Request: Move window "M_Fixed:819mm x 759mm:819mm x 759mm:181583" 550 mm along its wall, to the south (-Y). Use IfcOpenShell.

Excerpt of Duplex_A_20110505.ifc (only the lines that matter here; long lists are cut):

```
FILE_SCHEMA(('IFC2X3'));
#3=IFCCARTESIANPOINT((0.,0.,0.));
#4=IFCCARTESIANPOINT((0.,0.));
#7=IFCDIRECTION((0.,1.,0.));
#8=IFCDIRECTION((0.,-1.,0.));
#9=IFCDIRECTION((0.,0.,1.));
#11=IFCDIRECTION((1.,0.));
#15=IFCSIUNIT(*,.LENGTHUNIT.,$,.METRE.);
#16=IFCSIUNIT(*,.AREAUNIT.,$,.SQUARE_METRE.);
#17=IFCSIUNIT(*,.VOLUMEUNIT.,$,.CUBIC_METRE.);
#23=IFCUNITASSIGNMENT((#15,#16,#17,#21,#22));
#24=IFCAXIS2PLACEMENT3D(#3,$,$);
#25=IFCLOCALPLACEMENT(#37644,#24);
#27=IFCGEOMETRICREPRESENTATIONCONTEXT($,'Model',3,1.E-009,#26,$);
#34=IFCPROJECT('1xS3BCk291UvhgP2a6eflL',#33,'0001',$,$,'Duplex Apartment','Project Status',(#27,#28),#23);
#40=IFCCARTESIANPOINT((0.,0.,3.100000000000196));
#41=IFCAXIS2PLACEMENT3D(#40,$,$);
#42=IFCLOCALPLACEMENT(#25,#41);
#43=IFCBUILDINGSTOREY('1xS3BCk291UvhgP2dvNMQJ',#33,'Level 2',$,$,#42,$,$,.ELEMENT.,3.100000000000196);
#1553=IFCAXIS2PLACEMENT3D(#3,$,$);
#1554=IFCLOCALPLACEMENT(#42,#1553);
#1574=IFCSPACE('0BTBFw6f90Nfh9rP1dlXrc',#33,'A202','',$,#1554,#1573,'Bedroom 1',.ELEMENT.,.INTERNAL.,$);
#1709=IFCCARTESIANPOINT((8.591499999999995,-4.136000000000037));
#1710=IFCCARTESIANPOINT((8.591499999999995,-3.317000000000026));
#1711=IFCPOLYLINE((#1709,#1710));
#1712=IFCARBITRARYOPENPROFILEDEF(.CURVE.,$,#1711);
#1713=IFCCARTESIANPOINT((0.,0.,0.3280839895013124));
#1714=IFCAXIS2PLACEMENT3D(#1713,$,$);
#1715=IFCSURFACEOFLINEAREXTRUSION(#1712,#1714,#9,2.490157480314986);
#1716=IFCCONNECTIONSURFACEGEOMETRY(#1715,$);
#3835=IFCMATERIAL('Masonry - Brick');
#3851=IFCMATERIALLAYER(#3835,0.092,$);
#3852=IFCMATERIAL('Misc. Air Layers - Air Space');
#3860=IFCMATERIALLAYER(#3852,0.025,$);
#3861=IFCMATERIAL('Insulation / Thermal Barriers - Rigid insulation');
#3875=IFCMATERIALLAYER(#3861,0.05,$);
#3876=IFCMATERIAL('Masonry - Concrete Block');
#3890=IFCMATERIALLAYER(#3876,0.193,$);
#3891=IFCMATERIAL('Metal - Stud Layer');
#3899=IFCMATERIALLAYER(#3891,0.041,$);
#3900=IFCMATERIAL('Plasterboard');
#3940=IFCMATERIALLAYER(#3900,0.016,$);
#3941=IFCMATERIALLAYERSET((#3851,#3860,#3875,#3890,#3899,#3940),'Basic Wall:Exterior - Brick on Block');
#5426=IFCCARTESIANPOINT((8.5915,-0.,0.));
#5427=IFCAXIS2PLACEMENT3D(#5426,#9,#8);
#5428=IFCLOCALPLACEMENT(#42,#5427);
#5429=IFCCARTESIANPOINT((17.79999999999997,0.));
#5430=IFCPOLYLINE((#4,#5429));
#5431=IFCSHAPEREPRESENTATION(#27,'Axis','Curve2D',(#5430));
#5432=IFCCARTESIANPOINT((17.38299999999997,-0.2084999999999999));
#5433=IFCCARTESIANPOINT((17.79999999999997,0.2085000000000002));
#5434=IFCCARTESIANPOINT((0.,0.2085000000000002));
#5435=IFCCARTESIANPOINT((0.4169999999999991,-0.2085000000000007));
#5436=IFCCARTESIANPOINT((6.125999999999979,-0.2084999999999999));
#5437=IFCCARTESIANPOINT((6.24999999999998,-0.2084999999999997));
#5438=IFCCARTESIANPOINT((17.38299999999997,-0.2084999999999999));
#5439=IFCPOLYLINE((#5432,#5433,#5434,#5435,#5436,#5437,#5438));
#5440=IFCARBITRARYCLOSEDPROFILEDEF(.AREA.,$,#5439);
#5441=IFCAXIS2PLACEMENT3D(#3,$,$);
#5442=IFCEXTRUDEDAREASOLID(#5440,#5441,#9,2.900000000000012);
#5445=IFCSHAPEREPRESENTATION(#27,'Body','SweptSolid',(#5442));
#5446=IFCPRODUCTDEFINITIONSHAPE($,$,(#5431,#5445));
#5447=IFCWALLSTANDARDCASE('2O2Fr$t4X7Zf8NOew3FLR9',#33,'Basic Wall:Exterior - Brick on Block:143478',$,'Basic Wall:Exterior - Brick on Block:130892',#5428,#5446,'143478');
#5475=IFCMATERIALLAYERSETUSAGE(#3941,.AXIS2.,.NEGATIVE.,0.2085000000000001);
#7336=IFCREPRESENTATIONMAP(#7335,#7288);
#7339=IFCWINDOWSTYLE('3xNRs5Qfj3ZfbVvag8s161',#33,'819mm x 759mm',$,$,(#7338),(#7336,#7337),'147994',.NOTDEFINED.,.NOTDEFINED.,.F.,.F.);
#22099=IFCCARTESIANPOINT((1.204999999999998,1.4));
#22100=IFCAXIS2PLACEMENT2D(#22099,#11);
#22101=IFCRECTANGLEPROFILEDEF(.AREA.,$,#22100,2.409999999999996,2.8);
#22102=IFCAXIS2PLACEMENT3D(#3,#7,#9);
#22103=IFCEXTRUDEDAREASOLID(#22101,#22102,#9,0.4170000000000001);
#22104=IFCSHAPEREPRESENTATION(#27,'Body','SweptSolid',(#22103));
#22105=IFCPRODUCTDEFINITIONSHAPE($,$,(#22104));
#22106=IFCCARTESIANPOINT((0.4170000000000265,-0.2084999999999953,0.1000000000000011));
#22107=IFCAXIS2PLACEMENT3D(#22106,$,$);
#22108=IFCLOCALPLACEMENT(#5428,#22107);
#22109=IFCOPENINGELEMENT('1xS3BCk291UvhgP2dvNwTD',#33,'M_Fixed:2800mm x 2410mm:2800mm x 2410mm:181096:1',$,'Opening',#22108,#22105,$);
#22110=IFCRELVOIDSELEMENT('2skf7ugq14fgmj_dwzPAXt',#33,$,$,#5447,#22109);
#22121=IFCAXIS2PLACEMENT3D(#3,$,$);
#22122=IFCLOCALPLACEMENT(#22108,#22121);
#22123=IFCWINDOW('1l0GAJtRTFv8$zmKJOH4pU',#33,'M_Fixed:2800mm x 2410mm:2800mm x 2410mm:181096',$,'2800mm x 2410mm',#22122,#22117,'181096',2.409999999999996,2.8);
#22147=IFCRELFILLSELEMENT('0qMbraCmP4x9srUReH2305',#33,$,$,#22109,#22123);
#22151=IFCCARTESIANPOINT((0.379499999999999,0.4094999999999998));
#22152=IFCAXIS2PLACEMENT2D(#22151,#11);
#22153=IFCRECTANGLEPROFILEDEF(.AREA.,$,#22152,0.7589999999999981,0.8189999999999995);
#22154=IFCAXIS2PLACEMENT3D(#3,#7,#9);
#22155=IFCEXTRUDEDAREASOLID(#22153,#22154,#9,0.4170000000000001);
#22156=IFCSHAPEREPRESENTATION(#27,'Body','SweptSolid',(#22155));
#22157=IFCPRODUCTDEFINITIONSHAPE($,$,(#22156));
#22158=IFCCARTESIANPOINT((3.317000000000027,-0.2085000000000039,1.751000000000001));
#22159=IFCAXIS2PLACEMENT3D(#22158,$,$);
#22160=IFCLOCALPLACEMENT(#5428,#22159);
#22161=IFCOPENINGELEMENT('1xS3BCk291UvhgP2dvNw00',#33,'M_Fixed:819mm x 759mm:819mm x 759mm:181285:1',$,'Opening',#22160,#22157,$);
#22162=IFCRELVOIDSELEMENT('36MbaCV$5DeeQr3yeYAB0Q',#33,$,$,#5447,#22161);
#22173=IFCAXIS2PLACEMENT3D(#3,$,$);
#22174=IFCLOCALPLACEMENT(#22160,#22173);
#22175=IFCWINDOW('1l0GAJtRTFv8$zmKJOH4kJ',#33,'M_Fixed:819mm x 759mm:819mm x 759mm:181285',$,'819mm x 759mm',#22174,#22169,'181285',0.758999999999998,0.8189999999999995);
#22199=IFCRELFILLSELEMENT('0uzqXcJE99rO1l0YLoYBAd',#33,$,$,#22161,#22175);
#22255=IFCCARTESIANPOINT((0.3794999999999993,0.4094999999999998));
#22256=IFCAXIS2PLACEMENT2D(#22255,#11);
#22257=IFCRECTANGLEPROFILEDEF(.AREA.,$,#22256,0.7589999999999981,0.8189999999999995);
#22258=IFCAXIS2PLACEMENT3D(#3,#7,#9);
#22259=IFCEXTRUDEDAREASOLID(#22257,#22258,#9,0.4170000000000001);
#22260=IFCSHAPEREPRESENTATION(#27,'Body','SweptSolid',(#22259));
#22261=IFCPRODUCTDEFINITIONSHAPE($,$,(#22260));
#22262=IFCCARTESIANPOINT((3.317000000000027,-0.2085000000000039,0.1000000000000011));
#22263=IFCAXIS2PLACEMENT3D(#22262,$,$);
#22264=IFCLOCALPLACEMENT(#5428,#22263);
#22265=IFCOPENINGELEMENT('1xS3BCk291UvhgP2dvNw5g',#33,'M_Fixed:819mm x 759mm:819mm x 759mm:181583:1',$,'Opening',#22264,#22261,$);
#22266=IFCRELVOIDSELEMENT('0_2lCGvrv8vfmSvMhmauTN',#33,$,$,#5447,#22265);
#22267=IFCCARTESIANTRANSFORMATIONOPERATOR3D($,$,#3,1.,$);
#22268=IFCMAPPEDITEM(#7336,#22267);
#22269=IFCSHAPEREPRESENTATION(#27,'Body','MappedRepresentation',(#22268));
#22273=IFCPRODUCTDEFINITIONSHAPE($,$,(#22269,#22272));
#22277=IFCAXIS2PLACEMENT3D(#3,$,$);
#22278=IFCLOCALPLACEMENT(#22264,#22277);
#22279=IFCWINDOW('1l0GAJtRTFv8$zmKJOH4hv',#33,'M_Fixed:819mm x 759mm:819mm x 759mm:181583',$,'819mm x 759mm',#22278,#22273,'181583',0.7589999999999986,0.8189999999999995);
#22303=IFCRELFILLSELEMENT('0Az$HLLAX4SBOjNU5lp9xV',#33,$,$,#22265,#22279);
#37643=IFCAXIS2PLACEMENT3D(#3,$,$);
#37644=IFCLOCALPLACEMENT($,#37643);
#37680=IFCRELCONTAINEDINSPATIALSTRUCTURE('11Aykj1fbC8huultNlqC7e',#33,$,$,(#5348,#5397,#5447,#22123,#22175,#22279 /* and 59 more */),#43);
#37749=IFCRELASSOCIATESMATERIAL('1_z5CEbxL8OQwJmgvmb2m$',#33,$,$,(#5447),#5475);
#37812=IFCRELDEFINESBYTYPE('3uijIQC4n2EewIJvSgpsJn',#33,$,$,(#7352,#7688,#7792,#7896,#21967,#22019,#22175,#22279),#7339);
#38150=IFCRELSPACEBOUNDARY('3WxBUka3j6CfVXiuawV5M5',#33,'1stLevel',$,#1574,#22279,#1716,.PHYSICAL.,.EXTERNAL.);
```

```python
import numpy as np
import ifcopenshell
import ifcopenshell.api.geometry
import ifcopenshell.util.placement
import ifcopenshell.util.unit

model = ifcopenshell.open("Duplex_A_20110505.ifc")
unit_scale = ifcopenshell.util.unit.calculate_unit_scale(model)

window = model.by_id(22279)
opening = window.FillsVoids[0].RelatingOpeningElement
wall = opening.VoidsElements[0].RelatingBuildingElement

wall_matrix = ifcopenshell.util.placement.get_local_placement(wall.ObjectPlacement)
shift = wall_matrix[:3, 0] * 0.55 / unit_scale
before = ifcopenshell.util.placement.get_local_placement(window.ObjectPlacement)[:3, 3].copy()

# The window is placed relative to its opening, so it follows when the opening moves.
matrix = ifcopenshell.util.placement.get_local_placement(opening.ObjectPlacement)
matrix[:3, 3] += shift
ifcopenshell.api.geometry.edit_object_placement(
    model, product=opening, matrix=matrix, is_si=False, should_transform_children=True
)

# Space boundary surfaces are stored in each space's coordinates; move them too.
for rel in window.ProvidesBoundaries:
    if not rel.ConnectionGeometry:
        continue
    surface = rel.ConnectionGeometry.SurfaceOnRelatingElement
    space_matrix = ifcopenshell.util.placement.get_local_placement(rel.RelatingSpace.ObjectPlacement)
    point = np.array(surface.Position.Location.Coordinates) + space_matrix[:3, :3].T @ shift
    surface.Position = model.createIfcAxis2Placement3D(
        model.createIfcCartesianPoint(point.tolist()), surface.Position.Axis, surface.Position.RefDirection
    )

after = ifcopenshell.util.placement.get_local_placement(window.ObjectPlacement)[:3, 3]
print("window moved by", (after - before).round(3) + 0.0)

model.write("Duplex_A_20110505_edited.ifc")
```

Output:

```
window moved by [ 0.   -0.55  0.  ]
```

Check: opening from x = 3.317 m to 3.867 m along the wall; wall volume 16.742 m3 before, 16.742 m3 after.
